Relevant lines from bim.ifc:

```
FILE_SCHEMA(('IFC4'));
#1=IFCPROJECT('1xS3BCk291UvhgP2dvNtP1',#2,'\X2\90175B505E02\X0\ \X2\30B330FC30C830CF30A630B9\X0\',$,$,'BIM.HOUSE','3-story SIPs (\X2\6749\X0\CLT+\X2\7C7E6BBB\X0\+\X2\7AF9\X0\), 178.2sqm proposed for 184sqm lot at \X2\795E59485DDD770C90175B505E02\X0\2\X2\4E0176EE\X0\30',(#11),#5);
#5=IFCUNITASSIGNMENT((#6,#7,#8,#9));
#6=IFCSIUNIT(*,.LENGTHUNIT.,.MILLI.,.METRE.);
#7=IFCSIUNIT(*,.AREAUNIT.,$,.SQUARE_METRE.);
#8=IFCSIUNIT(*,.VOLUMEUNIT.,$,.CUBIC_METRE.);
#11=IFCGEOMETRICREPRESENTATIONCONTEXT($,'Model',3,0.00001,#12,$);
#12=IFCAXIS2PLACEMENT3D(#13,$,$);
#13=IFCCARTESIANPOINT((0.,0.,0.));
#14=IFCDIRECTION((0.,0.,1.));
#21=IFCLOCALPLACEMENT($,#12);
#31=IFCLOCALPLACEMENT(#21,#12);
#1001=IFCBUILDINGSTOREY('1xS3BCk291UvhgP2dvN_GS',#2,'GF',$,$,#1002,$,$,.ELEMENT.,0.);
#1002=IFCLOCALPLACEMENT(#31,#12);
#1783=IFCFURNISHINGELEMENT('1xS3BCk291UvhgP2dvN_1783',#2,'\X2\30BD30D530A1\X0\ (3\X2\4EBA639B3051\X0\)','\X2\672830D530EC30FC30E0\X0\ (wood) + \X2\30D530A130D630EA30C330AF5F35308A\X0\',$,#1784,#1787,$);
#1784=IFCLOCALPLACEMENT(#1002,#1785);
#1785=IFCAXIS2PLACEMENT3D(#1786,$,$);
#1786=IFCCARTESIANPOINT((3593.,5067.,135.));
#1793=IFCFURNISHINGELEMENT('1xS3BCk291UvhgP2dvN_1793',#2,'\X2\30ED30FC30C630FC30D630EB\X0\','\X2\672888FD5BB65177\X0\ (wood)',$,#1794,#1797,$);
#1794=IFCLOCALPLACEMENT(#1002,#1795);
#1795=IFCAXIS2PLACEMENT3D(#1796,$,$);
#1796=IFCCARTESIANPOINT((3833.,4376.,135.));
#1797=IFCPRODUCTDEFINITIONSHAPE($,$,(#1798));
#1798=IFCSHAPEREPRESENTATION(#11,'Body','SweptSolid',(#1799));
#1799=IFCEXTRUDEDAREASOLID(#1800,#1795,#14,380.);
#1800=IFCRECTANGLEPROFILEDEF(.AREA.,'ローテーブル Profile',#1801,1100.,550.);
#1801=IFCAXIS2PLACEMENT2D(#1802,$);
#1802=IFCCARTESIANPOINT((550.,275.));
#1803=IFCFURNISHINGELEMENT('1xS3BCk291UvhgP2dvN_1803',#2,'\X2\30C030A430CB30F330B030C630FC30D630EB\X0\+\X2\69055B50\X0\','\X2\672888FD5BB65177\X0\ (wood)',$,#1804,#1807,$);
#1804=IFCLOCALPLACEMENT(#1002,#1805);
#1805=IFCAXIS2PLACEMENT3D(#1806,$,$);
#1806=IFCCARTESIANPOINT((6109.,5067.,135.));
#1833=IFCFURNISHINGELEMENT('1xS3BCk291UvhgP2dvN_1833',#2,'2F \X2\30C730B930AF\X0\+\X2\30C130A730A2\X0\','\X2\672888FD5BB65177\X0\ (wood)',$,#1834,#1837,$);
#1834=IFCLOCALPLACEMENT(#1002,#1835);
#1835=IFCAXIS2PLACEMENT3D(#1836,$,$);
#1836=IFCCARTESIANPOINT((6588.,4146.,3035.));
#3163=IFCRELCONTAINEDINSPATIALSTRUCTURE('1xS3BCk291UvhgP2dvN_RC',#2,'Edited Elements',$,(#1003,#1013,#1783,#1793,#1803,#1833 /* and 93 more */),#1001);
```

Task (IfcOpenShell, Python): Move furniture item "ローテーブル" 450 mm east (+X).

```python
import ifcopenshell
import ifcopenshell.api.geometry
import ifcopenshell.util.placement
import ifcopenshell.util.unit

model = ifcopenshell.open("bim.ifc")
unit_scale = ifcopenshell.util.unit.calculate_unit_scale(model)

item = model.by_id(1793)
matrix = ifcopenshell.util.placement.get_local_placement(item.ObjectPlacement)
matrix[0, 3] += 0.45 / unit_scale
ifcopenshell.api.geometry.edit_object_placement(model, product=item, matrix=matrix, is_si=False)

print(ifcopenshell.util.placement.get_local_placement(item.ObjectPlacement).round(3) + 0.0)

model.write("bim_edited.ifc")
```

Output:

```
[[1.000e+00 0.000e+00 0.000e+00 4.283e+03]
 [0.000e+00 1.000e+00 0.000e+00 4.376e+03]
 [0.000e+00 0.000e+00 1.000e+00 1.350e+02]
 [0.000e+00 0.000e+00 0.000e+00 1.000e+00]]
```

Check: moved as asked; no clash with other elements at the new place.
